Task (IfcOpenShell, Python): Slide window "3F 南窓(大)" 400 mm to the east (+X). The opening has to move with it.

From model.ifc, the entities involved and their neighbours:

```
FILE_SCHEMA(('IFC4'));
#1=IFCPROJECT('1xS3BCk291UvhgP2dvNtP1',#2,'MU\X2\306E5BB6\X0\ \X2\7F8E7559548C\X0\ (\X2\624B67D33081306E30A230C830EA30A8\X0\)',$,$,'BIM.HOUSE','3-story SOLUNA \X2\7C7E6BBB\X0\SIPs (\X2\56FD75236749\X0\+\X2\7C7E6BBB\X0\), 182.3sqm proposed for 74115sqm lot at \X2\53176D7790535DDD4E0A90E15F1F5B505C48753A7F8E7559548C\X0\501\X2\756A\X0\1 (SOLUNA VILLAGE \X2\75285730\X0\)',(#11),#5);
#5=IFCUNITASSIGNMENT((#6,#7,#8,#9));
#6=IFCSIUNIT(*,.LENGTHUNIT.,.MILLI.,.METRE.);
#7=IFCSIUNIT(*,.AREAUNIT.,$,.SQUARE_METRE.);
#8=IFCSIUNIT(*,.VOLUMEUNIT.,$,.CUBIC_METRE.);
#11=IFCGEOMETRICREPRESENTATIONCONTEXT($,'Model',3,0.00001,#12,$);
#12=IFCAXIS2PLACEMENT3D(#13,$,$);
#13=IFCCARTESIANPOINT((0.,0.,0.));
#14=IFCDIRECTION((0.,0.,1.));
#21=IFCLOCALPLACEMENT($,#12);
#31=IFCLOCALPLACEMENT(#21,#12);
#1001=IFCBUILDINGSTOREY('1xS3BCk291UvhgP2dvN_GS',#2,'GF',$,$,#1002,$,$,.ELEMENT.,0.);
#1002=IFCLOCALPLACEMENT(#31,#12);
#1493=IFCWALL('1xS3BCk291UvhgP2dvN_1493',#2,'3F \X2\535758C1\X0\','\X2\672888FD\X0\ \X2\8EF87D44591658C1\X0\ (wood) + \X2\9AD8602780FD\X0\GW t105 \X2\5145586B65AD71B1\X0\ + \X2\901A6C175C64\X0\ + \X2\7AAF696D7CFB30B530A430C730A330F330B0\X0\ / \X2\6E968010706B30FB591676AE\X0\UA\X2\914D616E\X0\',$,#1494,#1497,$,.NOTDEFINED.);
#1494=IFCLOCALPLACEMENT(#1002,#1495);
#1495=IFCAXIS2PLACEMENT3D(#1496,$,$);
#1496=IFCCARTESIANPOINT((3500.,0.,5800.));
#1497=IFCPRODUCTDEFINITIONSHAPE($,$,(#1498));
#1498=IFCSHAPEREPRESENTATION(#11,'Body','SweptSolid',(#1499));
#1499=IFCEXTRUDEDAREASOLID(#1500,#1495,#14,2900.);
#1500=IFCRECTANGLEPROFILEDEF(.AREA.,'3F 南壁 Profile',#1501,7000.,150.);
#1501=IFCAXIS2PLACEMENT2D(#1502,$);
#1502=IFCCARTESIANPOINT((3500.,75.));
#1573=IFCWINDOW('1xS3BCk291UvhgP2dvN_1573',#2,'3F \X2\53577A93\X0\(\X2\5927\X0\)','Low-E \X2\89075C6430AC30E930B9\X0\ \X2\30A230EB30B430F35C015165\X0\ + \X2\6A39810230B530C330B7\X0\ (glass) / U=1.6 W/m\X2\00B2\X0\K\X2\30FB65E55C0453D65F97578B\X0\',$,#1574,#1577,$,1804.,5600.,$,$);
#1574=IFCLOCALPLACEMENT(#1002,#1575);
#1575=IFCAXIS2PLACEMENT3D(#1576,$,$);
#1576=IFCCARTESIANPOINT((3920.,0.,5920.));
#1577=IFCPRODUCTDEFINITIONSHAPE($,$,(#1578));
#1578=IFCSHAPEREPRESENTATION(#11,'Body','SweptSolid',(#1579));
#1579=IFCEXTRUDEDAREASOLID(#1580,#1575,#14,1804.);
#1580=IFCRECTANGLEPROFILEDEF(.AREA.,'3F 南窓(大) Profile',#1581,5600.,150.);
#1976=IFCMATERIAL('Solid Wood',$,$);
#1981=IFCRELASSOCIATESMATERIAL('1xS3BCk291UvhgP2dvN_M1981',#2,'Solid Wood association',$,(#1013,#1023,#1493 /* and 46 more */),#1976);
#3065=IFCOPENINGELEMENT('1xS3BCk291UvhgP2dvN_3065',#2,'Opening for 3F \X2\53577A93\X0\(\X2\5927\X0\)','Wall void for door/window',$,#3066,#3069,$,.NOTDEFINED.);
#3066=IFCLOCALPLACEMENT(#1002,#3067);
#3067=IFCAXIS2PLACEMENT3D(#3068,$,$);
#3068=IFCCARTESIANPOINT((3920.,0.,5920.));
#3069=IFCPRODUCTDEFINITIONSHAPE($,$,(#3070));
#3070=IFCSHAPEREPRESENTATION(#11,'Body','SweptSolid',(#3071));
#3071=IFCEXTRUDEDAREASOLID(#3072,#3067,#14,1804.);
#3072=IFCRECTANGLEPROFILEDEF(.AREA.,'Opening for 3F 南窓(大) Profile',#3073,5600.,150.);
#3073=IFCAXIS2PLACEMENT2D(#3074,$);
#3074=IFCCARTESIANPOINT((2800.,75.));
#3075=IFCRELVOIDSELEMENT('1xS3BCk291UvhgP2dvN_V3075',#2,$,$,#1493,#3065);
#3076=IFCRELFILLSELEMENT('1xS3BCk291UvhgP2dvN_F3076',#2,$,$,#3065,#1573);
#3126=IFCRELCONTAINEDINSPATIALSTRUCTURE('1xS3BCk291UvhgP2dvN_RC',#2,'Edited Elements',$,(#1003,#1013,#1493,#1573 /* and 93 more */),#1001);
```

```python
import ifcopenshell
import ifcopenshell.api.geometry
import ifcopenshell.util.placement
import ifcopenshell.util.unit

model = ifcopenshell.open("model.ifc")
unit_scale = ifcopenshell.util.unit.calculate_unit_scale(model)

window = model.by_id(1573)
opening = window.FillsVoids[0].RelatingOpeningElement
wall = opening.VoidsElements[0].RelatingBuildingElement

wall_matrix = ifcopenshell.util.placement.get_local_placement(wall.ObjectPlacement)
shift = wall_matrix[:3, 0] * 0.4 / unit_scale
before = ifcopenshell.util.placement.get_local_placement(window.ObjectPlacement)[:3, 3].copy()

# The window is not placed relative to its opening, so move both.
for product in (opening, window):
    matrix = ifcopenshell.util.placement.get_local_placement(product.ObjectPlacement)
    matrix[:3, 3] += shift
    ifcopenshell.api.geometry.edit_object_placement(model, product=product, matrix=matrix, is_si=False)

after = ifcopenshell.util.placement.get_local_placement(window.ObjectPlacement)[:3, 3]
print("window moved by", (after - before).round(3) + 0.0)

model.write("model-out.ifc")
```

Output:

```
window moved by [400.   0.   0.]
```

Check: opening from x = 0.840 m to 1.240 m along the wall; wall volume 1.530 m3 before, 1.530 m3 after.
